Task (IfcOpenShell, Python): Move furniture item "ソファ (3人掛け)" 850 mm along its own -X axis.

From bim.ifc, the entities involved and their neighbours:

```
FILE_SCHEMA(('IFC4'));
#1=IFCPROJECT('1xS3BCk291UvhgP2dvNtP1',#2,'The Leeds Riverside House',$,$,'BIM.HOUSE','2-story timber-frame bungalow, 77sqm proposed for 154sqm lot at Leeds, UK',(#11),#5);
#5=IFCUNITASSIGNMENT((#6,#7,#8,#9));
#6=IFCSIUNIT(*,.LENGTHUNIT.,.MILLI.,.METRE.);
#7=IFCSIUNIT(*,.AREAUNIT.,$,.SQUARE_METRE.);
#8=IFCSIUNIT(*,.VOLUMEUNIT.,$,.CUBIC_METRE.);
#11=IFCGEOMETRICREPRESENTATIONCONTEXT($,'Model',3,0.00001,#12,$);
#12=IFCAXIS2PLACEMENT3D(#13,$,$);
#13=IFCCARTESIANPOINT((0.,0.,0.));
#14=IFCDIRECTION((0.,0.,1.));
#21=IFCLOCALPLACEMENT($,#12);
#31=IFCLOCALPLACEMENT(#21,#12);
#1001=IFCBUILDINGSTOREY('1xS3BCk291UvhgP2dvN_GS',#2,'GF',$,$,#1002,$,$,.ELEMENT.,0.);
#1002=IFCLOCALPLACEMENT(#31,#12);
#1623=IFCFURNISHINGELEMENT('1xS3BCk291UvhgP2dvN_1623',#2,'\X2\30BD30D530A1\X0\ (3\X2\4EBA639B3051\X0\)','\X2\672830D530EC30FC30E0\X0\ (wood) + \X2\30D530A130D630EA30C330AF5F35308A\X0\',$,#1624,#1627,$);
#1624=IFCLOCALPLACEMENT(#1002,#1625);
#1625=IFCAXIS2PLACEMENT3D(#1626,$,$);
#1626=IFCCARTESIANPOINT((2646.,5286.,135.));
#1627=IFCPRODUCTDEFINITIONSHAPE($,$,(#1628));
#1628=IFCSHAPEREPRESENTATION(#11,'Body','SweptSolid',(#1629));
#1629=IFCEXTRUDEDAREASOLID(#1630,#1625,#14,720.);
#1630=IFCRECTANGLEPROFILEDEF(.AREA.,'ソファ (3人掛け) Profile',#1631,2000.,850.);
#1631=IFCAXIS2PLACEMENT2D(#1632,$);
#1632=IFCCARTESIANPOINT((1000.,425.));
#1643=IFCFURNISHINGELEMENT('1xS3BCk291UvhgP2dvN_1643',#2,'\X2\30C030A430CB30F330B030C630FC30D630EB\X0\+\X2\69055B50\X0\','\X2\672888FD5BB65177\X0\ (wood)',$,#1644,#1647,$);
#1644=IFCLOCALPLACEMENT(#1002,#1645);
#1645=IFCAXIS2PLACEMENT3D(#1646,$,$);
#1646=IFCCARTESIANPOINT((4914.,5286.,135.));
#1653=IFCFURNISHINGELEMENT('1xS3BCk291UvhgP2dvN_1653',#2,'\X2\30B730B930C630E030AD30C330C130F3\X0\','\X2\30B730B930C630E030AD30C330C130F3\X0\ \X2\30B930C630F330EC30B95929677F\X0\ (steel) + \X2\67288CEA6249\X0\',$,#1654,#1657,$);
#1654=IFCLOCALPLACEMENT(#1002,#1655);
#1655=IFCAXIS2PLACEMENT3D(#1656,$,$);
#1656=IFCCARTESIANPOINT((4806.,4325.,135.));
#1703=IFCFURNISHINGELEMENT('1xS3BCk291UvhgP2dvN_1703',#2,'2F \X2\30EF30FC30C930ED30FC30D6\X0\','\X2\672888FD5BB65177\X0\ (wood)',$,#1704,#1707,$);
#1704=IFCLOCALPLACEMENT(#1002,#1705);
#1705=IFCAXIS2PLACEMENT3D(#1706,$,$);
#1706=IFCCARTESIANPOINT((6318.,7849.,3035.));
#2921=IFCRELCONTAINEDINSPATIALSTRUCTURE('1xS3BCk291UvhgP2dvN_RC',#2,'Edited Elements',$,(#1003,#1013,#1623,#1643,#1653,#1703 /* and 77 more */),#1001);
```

```python
import ifcopenshell
import ifcopenshell.api.geometry
import ifcopenshell.util.placement
import ifcopenshell.util.unit

model = ifcopenshell.open("bim.ifc")
unit_scale = ifcopenshell.util.unit.calculate_unit_scale(model)

item = model.by_guid("1xS3BCk291UvhgP2dvN_1623")
matrix = ifcopenshell.util.placement.get_local_placement(item.ObjectPlacement)
matrix[:3, 3] -= matrix[:3, 0] * 0.85 / unit_scale
ifcopenshell.api.geometry.edit_object_placement(model, product=item, matrix=matrix, is_si=False)

print(ifcopenshell.util.placement.get_local_placement(item.ObjectPlacement).round(3) + 0.0)

model.write("bim_rev.ifc")
```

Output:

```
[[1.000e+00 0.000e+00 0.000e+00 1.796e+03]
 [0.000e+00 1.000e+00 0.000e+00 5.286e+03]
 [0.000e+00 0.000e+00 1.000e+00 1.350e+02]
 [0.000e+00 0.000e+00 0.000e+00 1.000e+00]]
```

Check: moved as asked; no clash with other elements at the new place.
